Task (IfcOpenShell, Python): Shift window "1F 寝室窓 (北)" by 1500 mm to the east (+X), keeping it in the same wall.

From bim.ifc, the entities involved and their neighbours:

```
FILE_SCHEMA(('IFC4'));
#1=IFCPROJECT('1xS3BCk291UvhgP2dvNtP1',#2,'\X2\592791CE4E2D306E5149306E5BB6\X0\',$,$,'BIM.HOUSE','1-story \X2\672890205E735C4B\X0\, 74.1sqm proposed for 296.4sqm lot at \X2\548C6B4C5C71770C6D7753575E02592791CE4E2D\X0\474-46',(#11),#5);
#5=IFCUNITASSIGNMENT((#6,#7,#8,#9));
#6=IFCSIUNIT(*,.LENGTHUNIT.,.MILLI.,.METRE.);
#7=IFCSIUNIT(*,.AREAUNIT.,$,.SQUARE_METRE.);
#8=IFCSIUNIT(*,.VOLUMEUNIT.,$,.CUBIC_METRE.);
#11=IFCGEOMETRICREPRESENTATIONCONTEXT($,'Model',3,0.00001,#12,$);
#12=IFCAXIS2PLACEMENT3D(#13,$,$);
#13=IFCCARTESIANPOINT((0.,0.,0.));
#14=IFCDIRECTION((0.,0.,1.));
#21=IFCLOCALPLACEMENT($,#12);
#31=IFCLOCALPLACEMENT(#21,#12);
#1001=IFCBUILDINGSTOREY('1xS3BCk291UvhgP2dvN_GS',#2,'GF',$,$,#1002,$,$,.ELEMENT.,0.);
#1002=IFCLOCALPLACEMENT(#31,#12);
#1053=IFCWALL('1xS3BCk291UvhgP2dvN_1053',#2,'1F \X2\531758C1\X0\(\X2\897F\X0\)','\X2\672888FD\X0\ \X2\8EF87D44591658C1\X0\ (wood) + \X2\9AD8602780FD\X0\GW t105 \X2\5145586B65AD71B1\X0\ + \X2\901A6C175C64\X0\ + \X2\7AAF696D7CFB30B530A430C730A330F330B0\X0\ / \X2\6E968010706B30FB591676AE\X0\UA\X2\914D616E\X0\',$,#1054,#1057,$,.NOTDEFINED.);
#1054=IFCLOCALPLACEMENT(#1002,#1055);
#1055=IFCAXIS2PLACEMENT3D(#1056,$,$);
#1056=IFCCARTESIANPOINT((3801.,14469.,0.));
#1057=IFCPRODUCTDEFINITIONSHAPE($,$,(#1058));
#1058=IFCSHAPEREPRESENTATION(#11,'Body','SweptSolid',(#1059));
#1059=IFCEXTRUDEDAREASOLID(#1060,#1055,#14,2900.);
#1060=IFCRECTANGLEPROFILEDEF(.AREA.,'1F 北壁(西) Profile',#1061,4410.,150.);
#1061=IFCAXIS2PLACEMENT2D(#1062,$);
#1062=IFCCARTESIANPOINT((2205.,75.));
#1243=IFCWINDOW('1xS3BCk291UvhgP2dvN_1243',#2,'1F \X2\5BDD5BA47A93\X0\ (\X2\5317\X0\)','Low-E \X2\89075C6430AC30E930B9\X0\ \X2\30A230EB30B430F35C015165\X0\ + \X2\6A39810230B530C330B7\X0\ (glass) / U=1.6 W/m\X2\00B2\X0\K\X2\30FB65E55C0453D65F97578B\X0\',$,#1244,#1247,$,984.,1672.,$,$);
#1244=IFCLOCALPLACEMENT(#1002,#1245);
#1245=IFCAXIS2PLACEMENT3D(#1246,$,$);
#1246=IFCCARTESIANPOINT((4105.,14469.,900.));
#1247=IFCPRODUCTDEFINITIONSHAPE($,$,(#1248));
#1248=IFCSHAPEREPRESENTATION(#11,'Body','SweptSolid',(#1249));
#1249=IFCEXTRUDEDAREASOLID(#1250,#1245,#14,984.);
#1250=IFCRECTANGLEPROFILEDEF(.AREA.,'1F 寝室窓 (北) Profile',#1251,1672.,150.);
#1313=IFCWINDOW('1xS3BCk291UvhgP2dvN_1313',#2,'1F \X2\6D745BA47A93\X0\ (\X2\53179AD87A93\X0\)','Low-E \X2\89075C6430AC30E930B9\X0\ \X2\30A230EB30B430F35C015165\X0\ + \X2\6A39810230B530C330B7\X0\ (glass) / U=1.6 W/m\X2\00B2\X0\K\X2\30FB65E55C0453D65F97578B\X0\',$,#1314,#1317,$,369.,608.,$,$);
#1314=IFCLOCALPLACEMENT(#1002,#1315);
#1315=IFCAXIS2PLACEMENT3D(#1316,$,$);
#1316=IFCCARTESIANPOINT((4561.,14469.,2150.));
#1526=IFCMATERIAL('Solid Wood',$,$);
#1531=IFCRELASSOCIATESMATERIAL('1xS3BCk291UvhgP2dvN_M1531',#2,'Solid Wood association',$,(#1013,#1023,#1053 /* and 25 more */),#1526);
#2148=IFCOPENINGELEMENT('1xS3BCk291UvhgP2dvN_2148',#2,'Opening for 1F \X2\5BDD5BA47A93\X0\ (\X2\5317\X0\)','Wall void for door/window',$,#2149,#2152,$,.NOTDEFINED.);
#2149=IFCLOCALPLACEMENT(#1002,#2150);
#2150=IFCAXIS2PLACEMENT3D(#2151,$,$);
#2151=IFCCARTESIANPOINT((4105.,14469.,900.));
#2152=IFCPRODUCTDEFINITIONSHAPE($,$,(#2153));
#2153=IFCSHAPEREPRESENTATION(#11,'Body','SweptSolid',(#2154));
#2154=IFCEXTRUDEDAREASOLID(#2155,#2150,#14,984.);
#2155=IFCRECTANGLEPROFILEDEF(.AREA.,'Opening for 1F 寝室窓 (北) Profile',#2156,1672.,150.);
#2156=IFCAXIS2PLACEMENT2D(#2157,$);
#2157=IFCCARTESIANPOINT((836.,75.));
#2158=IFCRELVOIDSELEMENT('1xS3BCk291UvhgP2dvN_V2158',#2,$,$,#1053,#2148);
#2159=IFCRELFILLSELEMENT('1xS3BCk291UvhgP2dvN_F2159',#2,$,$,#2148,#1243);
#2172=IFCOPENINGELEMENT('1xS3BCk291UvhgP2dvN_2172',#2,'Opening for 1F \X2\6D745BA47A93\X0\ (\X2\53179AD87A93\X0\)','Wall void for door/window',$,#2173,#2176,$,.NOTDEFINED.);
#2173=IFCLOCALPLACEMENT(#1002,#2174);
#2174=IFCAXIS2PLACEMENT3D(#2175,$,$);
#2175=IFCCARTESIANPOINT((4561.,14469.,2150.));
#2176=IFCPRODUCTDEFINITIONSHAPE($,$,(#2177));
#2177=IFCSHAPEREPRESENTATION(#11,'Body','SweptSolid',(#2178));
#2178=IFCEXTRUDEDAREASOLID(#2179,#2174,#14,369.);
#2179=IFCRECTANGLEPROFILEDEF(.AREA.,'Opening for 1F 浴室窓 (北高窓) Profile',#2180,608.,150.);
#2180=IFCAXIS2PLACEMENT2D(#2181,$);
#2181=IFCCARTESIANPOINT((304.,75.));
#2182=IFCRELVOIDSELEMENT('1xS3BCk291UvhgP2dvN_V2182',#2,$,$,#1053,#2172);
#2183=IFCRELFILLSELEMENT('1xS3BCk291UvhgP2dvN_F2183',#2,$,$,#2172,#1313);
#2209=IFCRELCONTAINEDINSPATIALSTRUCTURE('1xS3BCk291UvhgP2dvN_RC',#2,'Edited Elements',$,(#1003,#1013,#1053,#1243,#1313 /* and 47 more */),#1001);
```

```python
import ifcopenshell
import ifcopenshell.api.geometry
import ifcopenshell.util.placement

model = ifcopenshell.open("bim.ifc")

window = model.by_guid("1xS3BCk291UvhgP2dvN_1243")
opening = window.FillsVoids[0].RelatingOpeningElement
wall = opening.VoidsElements[0].RelatingBuildingElement

wall_matrix = ifcopenshell.util.placement.get_local_placement(wall.ObjectPlacement)
shift = wall_matrix[:3, 0] * 1500.0
before = ifcopenshell.util.placement.get_local_placement(window.ObjectPlacement)[:3, 3].copy()

# The window is not placed relative to its opening, so move both.
for product in (opening, window):
    matrix = ifcopenshell.util.placement.get_local_placement(product.ObjectPlacement)
    matrix[:3, 3] += shift
    ifcopenshell.api.geometry.edit_object_placement(model, product=product, matrix=matrix, is_si=False)

after = ifcopenshell.util.placement.get_local_placement(window.ObjectPlacement)[:3, 3]
print("window moved by", (after - before).round(3) + 0.0)

model.write("bim_rev.ifc")
```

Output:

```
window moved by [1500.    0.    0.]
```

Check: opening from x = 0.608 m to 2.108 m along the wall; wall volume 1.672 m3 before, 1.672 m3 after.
